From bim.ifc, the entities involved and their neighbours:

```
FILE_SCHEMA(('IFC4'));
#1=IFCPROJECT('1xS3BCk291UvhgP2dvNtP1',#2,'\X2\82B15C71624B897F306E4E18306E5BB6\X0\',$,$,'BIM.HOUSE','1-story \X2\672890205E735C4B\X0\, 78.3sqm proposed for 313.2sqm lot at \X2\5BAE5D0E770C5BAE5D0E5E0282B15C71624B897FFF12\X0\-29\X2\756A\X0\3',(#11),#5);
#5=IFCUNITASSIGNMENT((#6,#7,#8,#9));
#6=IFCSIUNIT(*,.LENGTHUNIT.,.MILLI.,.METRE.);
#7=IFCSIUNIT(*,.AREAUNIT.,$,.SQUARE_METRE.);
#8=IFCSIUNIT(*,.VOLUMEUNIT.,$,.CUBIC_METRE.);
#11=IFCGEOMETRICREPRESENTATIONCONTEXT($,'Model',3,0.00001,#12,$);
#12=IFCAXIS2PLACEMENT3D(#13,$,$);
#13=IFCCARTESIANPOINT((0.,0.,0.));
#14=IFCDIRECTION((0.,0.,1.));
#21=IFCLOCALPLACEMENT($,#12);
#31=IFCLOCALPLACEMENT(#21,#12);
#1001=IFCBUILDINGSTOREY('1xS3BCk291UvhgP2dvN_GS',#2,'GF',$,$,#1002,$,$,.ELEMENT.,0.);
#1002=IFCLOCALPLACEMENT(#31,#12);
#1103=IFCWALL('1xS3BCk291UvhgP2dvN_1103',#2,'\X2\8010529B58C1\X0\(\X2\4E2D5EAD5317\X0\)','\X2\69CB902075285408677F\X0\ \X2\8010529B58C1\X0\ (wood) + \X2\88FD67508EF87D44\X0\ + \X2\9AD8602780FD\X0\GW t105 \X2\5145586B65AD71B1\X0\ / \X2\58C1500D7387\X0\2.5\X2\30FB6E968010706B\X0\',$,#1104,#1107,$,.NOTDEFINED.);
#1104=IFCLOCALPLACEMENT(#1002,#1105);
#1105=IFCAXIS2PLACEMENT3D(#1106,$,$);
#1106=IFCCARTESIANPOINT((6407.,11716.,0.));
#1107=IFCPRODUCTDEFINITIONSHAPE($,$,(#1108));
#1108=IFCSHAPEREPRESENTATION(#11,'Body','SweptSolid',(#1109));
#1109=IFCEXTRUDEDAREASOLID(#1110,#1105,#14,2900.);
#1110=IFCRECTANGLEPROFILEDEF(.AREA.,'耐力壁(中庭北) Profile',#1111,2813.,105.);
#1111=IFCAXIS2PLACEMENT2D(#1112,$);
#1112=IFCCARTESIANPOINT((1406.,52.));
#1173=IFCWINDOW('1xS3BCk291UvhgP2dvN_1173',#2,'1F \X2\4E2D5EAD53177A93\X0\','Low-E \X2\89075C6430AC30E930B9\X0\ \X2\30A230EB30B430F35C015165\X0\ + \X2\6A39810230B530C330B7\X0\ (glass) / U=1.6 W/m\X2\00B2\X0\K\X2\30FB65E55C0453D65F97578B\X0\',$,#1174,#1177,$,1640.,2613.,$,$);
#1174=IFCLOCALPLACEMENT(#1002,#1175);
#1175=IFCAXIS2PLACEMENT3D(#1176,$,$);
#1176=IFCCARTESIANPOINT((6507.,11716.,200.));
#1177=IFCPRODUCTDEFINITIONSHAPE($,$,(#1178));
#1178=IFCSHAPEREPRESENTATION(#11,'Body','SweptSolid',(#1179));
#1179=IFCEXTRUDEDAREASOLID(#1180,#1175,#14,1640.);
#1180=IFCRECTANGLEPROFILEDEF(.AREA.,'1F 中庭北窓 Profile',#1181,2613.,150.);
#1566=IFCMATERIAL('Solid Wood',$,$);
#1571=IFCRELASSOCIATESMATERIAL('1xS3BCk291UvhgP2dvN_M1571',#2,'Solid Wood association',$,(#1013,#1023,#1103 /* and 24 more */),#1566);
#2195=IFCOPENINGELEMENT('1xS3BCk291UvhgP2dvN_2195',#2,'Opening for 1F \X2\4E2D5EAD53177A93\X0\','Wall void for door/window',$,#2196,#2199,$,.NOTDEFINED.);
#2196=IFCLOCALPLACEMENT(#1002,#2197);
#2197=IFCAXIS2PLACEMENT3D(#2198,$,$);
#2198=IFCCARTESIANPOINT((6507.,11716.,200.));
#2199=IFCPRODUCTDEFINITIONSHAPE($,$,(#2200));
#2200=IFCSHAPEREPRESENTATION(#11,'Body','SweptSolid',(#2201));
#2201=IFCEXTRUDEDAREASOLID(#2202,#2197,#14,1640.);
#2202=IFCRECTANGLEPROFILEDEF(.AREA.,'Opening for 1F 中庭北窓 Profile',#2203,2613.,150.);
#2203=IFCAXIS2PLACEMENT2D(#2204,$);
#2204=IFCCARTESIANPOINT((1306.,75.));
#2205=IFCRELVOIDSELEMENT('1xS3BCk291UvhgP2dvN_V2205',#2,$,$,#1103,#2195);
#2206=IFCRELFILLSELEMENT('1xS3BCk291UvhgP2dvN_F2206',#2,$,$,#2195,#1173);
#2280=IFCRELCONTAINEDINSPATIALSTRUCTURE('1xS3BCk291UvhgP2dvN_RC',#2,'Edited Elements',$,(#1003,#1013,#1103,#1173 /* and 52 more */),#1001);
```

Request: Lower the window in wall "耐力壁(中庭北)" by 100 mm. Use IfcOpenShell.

```python
import numpy as np
import ifcopenshell
import ifcopenshell.api.geometry
import ifcopenshell.util.placement
import ifcopenshell.util.unit

model = ifcopenshell.open("bim.ifc")
unit_scale = ifcopenshell.util.unit.calculate_unit_scale(model)

window = model.by_id(1173)
opening = window.FillsVoids[0].RelatingOpeningElement
dz = -0.1 / unit_scale

shift = np.array([0.0, 0.0, dz])
# The window is not placed relative to its opening, so move both.
for product in (opening, window):
    matrix = ifcopenshell.util.placement.get_local_placement(product.ObjectPlacement)
    matrix[:3, 3] += shift
    ifcopenshell.api.geometry.edit_object_placement(model, product=product, matrix=matrix, is_si=False)

print(f"moved by {dz * unit_scale:+.3f} m")

model.write("bim-out.ifc")
```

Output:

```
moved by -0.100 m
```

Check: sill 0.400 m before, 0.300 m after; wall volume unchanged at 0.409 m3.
